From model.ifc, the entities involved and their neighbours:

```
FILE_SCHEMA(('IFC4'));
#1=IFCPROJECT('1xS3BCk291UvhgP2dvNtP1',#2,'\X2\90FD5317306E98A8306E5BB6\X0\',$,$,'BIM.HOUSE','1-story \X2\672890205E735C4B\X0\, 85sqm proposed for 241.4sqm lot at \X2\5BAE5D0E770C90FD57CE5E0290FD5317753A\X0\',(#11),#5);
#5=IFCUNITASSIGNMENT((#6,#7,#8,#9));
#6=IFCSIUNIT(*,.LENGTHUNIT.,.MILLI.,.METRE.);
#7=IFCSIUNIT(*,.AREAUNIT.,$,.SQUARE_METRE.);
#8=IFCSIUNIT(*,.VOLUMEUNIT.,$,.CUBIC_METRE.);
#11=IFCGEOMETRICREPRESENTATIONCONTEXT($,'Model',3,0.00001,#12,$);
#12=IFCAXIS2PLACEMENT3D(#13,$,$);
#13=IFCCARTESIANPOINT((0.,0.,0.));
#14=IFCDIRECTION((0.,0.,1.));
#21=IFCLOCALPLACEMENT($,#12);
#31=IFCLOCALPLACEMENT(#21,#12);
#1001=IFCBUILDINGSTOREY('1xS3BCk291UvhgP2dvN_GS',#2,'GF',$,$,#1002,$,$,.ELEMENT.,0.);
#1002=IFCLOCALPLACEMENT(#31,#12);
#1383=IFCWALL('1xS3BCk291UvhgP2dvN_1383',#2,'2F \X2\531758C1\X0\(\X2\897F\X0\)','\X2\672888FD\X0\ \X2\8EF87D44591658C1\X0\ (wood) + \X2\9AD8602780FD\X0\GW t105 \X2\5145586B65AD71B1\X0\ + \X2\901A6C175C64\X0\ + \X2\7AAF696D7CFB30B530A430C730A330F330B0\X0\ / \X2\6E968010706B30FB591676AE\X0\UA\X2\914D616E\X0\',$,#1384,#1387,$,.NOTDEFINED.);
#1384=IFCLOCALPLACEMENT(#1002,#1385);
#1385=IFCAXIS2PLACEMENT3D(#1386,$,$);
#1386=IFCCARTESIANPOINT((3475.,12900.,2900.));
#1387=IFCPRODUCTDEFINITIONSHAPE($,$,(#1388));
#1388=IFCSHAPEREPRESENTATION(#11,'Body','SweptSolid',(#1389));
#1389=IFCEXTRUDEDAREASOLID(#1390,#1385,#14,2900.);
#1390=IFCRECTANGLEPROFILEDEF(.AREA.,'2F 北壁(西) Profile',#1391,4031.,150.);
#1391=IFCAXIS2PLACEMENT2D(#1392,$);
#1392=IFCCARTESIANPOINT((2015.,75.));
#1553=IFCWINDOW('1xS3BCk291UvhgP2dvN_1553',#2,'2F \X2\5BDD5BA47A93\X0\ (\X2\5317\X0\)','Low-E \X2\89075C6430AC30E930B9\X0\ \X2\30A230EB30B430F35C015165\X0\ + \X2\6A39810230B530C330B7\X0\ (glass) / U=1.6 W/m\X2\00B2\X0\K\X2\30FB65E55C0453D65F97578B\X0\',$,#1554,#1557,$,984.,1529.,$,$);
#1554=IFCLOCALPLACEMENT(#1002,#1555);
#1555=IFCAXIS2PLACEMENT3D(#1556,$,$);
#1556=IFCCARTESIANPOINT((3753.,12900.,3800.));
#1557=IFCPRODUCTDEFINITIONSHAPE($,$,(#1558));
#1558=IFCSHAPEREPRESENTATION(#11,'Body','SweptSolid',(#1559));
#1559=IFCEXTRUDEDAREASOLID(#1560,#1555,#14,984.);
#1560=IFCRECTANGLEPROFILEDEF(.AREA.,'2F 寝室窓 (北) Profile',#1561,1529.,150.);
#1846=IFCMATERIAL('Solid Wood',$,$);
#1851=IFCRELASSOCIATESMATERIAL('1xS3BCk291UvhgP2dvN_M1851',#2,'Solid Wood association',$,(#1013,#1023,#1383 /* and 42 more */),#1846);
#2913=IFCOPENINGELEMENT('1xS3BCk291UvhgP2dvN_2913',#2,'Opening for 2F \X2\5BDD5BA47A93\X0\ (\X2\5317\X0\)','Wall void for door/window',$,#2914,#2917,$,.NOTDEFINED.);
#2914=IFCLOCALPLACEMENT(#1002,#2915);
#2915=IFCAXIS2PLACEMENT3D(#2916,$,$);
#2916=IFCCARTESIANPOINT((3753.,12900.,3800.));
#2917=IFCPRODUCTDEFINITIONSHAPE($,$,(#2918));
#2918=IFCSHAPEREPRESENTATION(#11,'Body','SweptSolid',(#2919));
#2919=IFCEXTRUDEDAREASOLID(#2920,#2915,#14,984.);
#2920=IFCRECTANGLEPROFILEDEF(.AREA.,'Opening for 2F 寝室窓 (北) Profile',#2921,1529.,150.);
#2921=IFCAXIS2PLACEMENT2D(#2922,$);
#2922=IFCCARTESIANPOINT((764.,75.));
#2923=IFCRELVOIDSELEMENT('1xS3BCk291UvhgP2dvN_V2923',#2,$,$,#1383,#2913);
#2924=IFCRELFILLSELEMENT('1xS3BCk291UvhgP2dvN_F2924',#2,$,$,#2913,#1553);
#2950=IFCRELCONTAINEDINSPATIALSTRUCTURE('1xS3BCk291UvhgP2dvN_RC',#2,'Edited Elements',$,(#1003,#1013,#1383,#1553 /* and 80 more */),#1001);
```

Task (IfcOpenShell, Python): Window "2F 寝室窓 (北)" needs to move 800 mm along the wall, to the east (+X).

```python
import ifcopenshell
import ifcopenshell.api.geometry
import ifcopenshell.util.placement
import ifcopenshell.util.unit

model = ifcopenshell.open("model.ifc")
unit_scale = ifcopenshell.util.unit.calculate_unit_scale(model)

window = model.by_guid("1xS3BCk291UvhgP2dvN_1553")
opening = window.FillsVoids[0].RelatingOpeningElement
wall = opening.VoidsElements[0].RelatingBuildingElement

wall_matrix = ifcopenshell.util.placement.get_local_placement(wall.ObjectPlacement)
shift = wall_matrix[:3, 0] * 0.8 / unit_scale
before = ifcopenshell.util.placement.get_local_placement(window.ObjectPlacement)[:3, 3].copy()

# The window is not placed relative to its opening, so move both.
for product in (opening, window):
    matrix = ifcopenshell.util.placement.get_local_placement(product.ObjectPlacement)
    matrix[:3, 3] += shift
    ifcopenshell.api.geometry.edit_object_placement(model, product=product, matrix=matrix, is_si=False)

after = ifcopenshell.util.placement.get_local_placement(window.ObjectPlacement)[:3, 3]
print("window moved by", (after - before).round(3) + 0.0)

model.write("model_v2.ifc")
```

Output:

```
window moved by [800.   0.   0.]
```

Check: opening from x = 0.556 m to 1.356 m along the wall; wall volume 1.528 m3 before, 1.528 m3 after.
